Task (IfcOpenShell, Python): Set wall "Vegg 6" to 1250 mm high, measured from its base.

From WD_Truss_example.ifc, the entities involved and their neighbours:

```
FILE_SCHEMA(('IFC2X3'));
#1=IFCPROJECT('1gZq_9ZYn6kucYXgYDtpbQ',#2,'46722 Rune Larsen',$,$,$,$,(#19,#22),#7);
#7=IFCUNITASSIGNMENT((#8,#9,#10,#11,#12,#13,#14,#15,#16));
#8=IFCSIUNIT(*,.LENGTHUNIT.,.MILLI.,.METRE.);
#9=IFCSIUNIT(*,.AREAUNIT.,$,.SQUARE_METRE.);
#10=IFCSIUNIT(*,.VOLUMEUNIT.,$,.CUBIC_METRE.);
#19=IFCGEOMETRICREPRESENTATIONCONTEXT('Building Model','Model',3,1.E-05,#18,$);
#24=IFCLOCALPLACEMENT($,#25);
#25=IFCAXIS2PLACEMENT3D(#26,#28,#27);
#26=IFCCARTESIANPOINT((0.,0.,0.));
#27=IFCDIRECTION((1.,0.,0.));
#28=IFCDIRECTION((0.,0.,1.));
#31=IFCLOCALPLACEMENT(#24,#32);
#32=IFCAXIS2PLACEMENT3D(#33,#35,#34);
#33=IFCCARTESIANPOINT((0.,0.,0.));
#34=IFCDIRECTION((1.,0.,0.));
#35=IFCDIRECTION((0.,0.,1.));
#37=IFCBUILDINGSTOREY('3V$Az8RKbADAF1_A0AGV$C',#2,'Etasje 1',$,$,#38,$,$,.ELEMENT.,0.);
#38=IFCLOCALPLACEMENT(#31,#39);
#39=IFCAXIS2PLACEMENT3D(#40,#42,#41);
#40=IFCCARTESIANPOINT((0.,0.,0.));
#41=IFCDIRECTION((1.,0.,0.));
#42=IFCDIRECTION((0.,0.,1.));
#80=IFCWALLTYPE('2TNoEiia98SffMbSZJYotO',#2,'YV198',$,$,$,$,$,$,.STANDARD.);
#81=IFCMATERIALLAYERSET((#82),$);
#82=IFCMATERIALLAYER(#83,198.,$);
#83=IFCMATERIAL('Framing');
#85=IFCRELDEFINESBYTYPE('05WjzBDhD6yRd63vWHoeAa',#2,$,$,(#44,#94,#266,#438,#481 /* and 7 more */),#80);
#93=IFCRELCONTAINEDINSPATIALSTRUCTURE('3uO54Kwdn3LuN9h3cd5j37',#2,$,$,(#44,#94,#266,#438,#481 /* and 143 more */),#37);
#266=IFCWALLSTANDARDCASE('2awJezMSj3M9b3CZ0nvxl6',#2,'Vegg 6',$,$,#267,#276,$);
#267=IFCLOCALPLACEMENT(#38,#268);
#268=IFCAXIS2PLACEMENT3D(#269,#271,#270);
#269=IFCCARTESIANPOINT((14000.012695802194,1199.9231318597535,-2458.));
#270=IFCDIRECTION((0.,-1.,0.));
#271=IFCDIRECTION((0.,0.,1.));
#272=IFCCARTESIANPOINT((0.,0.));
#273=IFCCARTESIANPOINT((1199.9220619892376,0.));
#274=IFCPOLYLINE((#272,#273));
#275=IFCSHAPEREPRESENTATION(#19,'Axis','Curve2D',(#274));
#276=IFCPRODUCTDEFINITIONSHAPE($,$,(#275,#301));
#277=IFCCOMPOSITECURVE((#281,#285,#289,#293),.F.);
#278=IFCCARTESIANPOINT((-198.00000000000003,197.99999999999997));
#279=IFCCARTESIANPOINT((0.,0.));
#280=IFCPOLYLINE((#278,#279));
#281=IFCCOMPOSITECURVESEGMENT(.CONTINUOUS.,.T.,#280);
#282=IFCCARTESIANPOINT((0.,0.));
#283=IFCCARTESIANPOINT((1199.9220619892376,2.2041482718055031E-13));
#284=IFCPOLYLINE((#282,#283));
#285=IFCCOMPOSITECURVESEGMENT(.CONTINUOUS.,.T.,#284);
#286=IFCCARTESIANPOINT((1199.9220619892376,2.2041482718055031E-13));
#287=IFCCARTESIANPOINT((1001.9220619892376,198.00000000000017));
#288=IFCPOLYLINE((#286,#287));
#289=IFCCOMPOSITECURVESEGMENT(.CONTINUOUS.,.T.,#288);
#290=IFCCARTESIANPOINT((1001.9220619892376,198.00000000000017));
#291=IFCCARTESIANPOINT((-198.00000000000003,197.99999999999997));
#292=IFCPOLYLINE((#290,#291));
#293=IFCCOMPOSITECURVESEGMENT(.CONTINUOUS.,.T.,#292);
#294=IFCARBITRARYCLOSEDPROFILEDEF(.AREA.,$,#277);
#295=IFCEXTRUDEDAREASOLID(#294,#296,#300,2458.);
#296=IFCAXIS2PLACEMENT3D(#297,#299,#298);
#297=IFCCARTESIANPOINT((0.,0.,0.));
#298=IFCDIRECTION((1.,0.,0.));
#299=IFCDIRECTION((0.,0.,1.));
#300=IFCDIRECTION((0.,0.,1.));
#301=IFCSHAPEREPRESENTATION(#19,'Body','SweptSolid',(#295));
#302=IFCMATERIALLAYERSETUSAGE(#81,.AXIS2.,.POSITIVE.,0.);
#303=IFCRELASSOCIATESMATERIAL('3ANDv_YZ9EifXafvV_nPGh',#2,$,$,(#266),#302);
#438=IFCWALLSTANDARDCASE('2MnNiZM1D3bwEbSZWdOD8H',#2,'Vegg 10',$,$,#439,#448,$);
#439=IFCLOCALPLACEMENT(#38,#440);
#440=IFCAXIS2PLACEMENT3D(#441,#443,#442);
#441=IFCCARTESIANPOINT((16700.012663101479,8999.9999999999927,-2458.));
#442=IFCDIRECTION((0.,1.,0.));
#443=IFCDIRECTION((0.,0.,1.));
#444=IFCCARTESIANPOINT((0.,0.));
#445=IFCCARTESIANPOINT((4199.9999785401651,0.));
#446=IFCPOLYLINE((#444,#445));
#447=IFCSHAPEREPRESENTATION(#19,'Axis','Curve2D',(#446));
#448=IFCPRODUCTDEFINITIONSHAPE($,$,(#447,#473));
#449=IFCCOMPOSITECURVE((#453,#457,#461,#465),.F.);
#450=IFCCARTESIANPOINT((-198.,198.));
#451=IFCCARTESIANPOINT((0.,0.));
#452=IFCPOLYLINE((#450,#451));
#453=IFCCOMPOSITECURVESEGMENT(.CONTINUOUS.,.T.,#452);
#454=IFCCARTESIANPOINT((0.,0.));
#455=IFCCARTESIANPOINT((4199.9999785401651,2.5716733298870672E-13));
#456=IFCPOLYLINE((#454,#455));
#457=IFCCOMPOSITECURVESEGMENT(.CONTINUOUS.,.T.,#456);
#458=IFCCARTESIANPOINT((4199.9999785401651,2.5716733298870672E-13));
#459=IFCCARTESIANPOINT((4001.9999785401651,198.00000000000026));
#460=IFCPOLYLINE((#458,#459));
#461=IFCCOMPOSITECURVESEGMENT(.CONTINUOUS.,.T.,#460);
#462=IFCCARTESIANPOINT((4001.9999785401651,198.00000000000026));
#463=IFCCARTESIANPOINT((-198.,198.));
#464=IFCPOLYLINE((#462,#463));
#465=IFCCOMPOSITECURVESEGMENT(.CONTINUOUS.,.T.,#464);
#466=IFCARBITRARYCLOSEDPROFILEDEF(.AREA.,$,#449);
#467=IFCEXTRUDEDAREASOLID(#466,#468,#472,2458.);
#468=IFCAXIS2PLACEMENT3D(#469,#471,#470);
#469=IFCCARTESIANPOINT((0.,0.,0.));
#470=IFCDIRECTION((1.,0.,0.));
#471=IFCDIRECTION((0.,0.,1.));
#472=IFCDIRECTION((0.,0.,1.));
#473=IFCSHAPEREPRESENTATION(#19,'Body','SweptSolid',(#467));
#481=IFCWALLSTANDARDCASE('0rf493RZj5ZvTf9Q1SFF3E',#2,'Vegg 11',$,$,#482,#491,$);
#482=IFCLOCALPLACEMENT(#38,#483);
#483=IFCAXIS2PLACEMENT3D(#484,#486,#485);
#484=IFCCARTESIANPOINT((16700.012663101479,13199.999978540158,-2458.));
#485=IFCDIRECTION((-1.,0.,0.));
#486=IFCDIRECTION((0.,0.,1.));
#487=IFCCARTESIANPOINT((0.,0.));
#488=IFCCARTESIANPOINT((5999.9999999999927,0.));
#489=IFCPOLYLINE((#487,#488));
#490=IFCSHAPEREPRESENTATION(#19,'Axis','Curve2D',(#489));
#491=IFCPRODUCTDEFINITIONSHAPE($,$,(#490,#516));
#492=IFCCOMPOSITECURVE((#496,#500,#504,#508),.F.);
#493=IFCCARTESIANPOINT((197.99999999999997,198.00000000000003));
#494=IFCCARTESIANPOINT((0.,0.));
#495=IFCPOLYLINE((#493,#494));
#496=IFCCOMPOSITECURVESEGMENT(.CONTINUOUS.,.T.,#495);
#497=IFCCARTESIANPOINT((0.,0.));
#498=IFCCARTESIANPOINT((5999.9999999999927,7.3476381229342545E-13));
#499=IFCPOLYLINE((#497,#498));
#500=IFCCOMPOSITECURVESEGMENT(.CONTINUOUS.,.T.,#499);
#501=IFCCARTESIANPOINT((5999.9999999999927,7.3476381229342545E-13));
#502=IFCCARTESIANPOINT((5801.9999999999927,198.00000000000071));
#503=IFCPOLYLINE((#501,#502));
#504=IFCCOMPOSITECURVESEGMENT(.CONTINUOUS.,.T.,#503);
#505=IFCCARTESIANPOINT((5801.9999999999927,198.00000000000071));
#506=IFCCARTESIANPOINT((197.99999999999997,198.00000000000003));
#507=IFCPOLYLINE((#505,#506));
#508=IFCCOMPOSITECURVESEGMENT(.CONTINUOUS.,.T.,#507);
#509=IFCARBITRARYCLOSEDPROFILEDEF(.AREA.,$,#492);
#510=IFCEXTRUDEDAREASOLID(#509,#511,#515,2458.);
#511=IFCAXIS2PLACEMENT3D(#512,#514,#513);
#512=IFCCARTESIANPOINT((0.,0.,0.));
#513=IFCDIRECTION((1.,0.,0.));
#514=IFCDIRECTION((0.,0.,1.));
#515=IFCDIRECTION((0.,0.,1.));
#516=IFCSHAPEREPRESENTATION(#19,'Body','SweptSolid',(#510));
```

```python
import ifcopenshell
import ifcopenshell.geom
import ifcopenshell.util.shape

model = ifcopenshell.open("WD_Truss_example.ifc")
settings = ifcopenshell.geom.settings()


def volume(element):
    """Net volume in cubic metres, openings subtracted."""
    shape = ifcopenshell.geom.create_shape(settings, element)
    return ifcopenshell.util.shape.get_volume(shape.geometry)


wall = model.by_guid("2awJezMSj3M9b3CZ0nvxl6")
before = volume(wall)

body = next(r for r in wall.Representation.Representations if r.RepresentationIdentifier == "Body")
solid = body.Items[0]
old_height = solid.Depth
solid.Depth = 1250.0
after = volume(wall)

print(f"height {old_height:g} -> {solid.Depth:g}, volume {before:.3f} -> {after:.3f} m3")

model.write("WD_Truss_example_edited.ifc")
```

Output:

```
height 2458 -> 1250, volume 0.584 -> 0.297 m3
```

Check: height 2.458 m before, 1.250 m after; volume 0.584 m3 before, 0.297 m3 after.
